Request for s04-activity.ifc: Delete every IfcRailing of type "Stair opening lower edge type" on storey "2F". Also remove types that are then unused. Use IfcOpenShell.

First a look at what the model holds.

```python
import ifcopenshell
import ifcopenshell.util.element

model = ifcopenshell.open("s04-activity.ifc")
print(model.schema)
storey = next(s for s in model.by_type("IfcBuildingStorey") if s.Name == "2F")
railings = [e for e in ifcopenshell.util.element.get_decomposition(storey) if e.is_a("IfcRailing")]
seen = {}
for e in railings:
    element_type = ifcopenshell.util.element.get_type(e)
    name = element_type.Name if element_type not in (None, e) else None
    seen[name] = seen.get(name, 0) + 1
for name, count in sorted(seen.items(), key=str):
    print(count, "x", name)
```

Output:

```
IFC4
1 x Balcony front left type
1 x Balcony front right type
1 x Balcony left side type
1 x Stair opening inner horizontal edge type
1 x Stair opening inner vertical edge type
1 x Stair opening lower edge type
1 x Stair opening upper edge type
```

```python
import ifcopenshell
import ifcopenshell.api.root
import ifcopenshell.util.element

model = ifcopenshell.open("s04-activity.ifc")

storey = next(s for s in model.by_type("IfcBuildingStorey") if s.Name == "2F")
railings = [e for e in ifcopenshell.util.element.get_decomposition(storey) if e.is_a("IfcRailing")]
targets = [e for e in railings if (t := ifcopenshell.util.element.get_type(e)) not in (None, e) and t.Name == "Stair opening lower edge type"]
types = {ifcopenshell.util.element.get_type(e) for e in targets} - {None, *targets}

for e in targets:
    ifcopenshell.api.root.remove_product(model, product=e)
print(len(targets), "removed")

unused = [t for t in types if not ifcopenshell.util.element.get_types(t)]
for t in unused:
    ifcopenshell.api.root.remove_product(model, product=t)
print(len(unused), "unused types removed")

model.write("s04-activity-out.ifc")
```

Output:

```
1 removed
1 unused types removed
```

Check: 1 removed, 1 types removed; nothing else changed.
